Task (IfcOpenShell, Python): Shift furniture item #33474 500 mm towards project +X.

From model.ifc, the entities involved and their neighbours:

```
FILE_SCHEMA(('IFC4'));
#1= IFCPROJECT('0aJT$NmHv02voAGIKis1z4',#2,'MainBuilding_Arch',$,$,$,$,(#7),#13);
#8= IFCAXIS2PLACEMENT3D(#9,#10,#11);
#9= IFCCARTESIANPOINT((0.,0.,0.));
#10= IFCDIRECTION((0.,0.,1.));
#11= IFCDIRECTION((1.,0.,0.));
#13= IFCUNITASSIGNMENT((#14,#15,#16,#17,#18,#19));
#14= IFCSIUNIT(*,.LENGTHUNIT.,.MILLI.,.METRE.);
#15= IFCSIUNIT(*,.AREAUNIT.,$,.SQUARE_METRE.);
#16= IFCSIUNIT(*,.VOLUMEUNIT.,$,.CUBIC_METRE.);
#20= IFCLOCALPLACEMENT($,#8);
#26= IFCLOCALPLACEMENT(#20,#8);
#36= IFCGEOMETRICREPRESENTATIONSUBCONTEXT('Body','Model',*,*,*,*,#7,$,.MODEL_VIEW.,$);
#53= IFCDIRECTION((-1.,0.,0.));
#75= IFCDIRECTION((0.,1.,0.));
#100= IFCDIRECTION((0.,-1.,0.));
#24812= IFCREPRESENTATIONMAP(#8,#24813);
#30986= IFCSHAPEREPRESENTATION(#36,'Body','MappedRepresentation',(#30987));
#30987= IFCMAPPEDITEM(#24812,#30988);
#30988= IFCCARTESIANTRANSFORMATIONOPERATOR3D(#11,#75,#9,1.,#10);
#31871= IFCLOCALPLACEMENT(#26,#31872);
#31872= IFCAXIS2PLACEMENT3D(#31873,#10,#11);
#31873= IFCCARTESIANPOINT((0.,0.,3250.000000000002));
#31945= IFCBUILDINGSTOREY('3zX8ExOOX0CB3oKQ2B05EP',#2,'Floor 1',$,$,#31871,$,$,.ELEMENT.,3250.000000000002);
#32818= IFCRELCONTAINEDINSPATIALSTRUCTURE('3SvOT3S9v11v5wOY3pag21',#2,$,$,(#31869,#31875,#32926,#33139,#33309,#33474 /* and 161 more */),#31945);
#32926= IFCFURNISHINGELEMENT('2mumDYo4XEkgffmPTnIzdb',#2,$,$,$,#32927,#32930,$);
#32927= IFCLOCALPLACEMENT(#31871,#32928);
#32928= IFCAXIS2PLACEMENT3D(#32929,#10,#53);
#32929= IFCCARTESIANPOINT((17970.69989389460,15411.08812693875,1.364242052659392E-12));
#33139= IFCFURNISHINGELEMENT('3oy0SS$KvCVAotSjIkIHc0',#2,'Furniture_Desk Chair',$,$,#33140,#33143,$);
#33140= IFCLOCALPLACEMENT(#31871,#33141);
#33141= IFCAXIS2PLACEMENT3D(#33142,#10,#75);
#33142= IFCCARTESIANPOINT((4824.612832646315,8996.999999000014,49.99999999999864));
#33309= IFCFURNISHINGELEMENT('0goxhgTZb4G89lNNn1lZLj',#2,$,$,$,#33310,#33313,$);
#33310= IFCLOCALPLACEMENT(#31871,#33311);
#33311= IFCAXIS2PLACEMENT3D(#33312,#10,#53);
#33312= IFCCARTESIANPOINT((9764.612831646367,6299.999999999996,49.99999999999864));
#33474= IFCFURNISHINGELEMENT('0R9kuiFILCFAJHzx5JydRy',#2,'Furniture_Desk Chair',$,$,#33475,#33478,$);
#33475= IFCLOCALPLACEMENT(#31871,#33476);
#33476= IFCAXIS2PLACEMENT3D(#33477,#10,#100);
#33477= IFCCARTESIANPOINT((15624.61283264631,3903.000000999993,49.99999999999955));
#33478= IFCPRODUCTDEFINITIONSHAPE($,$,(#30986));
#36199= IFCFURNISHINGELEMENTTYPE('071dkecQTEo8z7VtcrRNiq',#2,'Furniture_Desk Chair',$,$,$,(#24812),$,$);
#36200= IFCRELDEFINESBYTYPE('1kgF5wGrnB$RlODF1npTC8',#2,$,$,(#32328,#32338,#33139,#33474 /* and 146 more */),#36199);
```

```python
import ifcopenshell
import ifcopenshell.api.geometry
import ifcopenshell.util.placement

model = ifcopenshell.open("model.ifc")

item = model.by_id(33474)
matrix = ifcopenshell.util.placement.get_local_placement(item.ObjectPlacement)
matrix[0, 3] += 500.0
ifcopenshell.api.geometry.edit_object_placement(model, product=item, matrix=matrix, is_si=False)

print(ifcopenshell.util.placement.get_local_placement(item.ObjectPlacement).round(3) + 0.0)

model.write("model_updated.ifc")
```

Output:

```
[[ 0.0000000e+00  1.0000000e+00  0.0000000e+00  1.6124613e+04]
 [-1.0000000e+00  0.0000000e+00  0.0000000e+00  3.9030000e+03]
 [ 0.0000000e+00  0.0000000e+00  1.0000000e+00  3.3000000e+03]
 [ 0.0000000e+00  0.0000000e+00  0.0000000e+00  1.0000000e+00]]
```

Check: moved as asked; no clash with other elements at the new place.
